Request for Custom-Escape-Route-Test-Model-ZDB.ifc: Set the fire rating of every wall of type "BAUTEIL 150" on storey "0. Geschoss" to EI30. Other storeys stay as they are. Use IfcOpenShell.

First a look at what the model holds.

```python
import ifcopenshell
import ifcopenshell.util.element

model = ifcopenshell.open("Custom-Escape-Route-Test-Model-ZDB.ifc")
print(model.schema)
storey = next(s for s in model.by_type("IfcBuildingStorey") if s.Name == "0. Geschoss")
walls = [e for e in ifcopenshell.util.element.get_decomposition(storey) if e.is_a("IfcWall")]
seen = {}
for e in walls:
    element_type = ifcopenshell.util.element.get_type(e)
    key = (element_type.Name if element_type != e and element_type else None, ifcopenshell.util.element.get_pset(e, "Pset_WallCommon", "FireRating"))
    seen[key] = seen.get(key, 0) + 1
for (name, value), count in sorted(seen.items(), key=str):
    print(count, "x", name, "|", value)
```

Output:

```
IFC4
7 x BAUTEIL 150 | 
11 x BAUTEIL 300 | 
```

```python
import ifcopenshell
import ifcopenshell.api.pset
import ifcopenshell.util.element

model = ifcopenshell.open("Custom-Escape-Route-Test-Model-ZDB.ifc")

storey = next(s for s in model.by_type("IfcBuildingStorey") if s.Name == "0. Geschoss")
walls = [e for e in ifcopenshell.util.element.get_decomposition(storey) if e.is_a("IfcWall")]

count = 0
for e in walls:
    element_type = ifcopenshell.util.element.get_type(e)
    if element_type in (None, e) or element_type.Name != "BAUTEIL 150":
        continue
    # add_pset returns the element's existing set when there is one.
    pset = ifcopenshell.api.pset.add_pset(model, product=e, name="Pset_WallCommon")
    ifcopenshell.api.pset.edit_pset(model, pset=pset, properties={"FireRating": "EI30"})
    count += 1

print(count, "walls updated")

model.write("Custom-Escape-Route-Test-Model-ZDB_edited.ifc")
```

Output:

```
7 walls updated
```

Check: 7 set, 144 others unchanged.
